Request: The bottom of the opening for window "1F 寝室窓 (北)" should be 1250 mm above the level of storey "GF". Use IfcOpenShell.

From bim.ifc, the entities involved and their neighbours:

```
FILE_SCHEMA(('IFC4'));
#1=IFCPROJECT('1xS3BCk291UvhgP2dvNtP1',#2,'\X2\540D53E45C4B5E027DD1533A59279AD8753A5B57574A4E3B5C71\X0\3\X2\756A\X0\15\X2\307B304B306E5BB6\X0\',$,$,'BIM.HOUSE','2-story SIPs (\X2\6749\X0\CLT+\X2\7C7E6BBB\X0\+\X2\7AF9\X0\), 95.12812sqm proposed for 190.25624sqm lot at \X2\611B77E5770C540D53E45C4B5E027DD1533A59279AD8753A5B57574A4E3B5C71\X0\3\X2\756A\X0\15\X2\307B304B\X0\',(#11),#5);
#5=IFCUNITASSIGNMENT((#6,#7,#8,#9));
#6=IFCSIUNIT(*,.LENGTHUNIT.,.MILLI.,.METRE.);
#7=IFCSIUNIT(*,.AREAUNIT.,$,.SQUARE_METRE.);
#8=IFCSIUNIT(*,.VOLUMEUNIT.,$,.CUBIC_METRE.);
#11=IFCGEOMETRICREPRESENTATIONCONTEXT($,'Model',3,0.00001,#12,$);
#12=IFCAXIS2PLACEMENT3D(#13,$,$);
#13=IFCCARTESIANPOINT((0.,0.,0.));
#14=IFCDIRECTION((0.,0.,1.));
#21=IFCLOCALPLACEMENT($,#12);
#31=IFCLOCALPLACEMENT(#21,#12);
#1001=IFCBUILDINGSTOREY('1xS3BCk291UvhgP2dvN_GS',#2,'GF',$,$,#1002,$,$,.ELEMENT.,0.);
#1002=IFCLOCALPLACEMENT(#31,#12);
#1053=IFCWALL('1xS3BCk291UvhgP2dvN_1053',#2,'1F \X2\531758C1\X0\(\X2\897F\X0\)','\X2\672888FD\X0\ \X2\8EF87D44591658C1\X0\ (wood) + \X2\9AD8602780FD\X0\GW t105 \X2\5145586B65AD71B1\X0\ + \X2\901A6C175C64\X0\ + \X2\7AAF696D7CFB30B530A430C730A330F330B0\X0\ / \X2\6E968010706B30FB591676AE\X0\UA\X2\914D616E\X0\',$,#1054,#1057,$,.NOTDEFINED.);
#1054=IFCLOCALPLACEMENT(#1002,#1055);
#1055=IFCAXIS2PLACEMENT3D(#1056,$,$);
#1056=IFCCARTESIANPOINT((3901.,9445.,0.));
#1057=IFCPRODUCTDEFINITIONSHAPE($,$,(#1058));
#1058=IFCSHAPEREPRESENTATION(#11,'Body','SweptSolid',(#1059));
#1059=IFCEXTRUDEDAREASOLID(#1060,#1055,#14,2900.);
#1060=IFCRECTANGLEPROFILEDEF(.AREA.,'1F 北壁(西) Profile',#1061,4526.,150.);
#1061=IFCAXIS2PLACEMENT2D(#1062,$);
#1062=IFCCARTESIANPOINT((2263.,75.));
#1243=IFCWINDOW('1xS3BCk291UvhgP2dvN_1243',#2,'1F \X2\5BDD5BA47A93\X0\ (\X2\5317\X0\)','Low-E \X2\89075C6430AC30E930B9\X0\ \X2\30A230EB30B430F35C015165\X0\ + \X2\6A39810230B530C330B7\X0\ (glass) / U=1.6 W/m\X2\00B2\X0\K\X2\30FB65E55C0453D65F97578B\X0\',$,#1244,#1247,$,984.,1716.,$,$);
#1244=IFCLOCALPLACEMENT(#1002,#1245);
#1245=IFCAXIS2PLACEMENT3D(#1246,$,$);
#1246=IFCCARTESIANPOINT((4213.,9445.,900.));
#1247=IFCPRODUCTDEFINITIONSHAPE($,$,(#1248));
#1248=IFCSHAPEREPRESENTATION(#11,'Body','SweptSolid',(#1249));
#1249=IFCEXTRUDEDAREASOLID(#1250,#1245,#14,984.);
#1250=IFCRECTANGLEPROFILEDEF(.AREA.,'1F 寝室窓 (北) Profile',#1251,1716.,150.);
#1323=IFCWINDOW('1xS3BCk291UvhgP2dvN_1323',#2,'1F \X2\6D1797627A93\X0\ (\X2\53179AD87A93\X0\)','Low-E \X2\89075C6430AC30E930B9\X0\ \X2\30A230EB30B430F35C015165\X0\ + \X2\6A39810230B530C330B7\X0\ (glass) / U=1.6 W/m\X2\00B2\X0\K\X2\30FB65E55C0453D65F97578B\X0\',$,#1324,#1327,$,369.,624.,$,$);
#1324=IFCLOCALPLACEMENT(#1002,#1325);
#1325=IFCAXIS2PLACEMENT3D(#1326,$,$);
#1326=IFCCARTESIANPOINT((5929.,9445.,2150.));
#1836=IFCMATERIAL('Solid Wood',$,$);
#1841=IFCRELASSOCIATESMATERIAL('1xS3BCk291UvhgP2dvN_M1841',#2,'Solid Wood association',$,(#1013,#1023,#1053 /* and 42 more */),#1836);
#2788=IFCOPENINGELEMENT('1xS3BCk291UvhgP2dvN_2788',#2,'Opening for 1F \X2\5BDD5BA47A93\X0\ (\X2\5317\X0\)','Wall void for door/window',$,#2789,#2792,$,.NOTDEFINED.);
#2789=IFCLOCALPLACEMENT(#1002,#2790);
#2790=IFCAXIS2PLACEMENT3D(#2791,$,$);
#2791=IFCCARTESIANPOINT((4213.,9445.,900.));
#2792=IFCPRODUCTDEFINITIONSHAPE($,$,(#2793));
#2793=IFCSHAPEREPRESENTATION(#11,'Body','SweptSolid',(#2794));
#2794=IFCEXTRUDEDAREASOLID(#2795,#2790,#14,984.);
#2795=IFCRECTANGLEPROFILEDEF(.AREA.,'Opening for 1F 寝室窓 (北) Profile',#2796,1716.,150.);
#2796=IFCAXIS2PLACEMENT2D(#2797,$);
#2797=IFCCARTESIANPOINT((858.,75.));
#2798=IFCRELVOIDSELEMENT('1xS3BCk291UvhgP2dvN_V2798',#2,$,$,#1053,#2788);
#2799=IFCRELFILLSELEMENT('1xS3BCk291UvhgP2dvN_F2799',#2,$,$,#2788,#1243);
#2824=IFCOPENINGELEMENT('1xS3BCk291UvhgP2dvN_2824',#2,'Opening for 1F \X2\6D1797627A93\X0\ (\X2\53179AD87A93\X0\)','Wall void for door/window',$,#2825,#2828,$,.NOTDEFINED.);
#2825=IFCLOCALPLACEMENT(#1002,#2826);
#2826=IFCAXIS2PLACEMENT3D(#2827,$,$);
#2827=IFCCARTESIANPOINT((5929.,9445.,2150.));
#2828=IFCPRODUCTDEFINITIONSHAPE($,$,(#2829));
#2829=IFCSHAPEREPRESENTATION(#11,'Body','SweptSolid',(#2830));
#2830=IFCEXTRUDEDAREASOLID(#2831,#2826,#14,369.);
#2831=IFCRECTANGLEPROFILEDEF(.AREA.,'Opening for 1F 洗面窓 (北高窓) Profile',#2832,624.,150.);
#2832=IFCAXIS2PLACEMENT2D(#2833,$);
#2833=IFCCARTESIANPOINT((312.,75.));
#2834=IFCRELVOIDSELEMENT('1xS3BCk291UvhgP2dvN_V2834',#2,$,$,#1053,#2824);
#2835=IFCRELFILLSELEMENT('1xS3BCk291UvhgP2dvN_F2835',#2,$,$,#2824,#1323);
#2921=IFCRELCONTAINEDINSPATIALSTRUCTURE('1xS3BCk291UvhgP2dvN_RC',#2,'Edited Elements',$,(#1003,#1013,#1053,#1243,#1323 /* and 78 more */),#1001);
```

```python
import numpy as np
import ifcopenshell
import ifcopenshell.api.geometry
import ifcopenshell.geom
import ifcopenshell.util.element
import ifcopenshell.util.placement
import ifcopenshell.util.shape
import ifcopenshell.util.unit

model = ifcopenshell.open("bim.ifc")
unit_scale = ifcopenshell.util.unit.calculate_unit_scale(model)

window = model.by_guid("1xS3BCk291UvhgP2dvN_1243")
opening = window.FillsVoids[0].RelatingOpeningElement
storey = ifcopenshell.util.element.get_container(window, ifc_class="IfcBuildingStorey")
level = ifcopenshell.util.placement.get_local_placement(storey.ObjectPlacement)[2, 3]

# The opening's origin need not be at the sill, so measure its lowest point.
shape = ifcopenshell.geom.create_shape(ifcopenshell.geom.settings(), opening)
bottom = ifcopenshell.util.shape.get_shape_bottom_elevation(shape, shape.geometry) / unit_scale
dz = level + 1.25 / unit_scale - bottom

shift = np.array([0.0, 0.0, dz])
# The window is not placed relative to its opening, so move both.
for product in (opening, window):
    matrix = ifcopenshell.util.placement.get_local_placement(product.ObjectPlacement)
    matrix[:3, 3] += shift
    ifcopenshell.api.geometry.edit_object_placement(model, product=product, matrix=matrix, is_si=False)

print(f"moved by {dz * unit_scale:+.3f} m")

model.write("bim-out.ifc")
```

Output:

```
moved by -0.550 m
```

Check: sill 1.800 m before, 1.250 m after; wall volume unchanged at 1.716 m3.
